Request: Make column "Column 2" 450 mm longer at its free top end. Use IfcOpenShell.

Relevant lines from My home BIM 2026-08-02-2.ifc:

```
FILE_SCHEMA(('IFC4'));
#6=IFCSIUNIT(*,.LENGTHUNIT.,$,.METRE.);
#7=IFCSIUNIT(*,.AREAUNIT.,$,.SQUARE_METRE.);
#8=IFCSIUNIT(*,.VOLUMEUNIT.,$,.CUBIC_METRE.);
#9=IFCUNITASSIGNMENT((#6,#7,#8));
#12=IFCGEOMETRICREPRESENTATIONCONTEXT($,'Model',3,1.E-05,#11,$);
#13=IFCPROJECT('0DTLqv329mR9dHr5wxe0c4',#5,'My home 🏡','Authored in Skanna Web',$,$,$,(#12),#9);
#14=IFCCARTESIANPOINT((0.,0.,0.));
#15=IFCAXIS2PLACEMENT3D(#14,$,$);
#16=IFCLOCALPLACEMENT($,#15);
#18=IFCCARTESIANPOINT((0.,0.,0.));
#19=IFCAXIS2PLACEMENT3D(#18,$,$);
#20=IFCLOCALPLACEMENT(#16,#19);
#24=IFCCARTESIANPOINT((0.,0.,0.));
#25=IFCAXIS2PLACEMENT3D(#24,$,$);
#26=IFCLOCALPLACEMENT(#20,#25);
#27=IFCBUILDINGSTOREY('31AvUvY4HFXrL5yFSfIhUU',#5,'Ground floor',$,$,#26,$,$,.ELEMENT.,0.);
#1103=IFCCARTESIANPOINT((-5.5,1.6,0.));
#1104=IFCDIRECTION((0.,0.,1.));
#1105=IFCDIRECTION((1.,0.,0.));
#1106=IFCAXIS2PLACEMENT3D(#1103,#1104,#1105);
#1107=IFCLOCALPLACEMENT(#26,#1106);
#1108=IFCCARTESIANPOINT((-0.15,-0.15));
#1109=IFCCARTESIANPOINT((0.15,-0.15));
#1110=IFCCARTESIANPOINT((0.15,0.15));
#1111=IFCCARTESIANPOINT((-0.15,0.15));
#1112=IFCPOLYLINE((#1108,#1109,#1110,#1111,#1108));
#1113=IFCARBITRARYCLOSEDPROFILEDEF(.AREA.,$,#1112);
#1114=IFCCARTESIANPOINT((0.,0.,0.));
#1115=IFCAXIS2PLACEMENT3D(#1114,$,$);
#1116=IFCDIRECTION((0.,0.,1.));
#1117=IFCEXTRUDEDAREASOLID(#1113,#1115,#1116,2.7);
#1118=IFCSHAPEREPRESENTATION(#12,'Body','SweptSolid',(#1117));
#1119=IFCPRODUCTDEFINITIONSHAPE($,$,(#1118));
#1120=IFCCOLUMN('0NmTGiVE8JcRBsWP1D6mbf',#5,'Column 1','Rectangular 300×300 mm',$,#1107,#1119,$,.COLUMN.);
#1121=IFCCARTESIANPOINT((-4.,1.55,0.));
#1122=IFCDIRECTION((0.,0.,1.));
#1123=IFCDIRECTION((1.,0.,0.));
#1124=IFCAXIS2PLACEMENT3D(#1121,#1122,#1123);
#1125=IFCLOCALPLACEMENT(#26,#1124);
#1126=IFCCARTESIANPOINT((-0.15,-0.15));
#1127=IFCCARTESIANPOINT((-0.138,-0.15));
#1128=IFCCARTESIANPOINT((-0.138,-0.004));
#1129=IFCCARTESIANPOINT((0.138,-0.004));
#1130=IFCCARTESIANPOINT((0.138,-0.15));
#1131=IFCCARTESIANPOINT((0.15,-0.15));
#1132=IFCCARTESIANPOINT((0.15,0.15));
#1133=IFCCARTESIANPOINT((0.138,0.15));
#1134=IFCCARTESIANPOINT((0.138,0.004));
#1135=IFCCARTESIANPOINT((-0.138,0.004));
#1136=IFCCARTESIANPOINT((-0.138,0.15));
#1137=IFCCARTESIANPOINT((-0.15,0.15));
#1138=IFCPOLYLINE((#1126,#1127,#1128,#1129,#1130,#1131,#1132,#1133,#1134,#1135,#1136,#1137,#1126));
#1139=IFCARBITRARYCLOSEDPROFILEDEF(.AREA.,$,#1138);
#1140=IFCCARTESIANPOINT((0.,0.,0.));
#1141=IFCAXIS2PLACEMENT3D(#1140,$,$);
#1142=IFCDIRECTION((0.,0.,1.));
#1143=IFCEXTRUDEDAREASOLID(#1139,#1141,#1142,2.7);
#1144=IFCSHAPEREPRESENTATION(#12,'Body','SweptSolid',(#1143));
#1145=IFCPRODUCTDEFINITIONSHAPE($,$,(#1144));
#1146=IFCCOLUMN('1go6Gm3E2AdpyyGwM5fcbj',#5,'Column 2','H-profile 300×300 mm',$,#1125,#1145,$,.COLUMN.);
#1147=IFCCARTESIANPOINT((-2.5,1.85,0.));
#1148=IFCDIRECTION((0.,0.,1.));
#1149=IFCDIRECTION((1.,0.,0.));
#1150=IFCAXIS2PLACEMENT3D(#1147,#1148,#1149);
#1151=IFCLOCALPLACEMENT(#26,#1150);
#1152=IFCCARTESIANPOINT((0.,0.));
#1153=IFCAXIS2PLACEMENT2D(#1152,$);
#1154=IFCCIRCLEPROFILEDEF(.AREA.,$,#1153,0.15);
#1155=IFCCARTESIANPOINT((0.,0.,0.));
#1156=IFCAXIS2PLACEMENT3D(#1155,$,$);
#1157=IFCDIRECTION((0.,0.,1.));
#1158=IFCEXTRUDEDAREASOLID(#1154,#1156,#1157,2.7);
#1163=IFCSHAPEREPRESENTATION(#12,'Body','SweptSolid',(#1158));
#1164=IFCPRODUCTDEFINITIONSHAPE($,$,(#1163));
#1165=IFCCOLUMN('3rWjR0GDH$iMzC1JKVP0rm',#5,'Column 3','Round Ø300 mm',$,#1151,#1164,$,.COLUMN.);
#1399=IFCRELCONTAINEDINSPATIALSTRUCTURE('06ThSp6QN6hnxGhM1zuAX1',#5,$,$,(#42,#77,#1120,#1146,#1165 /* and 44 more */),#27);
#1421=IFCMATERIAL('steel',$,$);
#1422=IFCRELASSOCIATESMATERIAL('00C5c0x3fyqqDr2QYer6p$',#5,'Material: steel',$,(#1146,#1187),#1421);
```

```python
import ifcopenshell
import ifcopenshell.util.unit

model = ifcopenshell.open("My home BIM 2026-08-02-2.ifc")
unit_scale = ifcopenshell.util.unit.calculate_unit_scale(model)

member = model.by_id(1146)
change = 0.45 / unit_scale

# The extrusion runs towards the end named, so only its depth changes.
body = next(r for r in member.Representation.Representations if r.RepresentationIdentifier == "Body")
solid = body.Items[0]
old_length = solid.Depth
solid.Depth += change

print(f"length {old_length:g} -> {solid.Depth:g}")

model.write("My home BIM 2026-08-02-2_rev.ifc")
```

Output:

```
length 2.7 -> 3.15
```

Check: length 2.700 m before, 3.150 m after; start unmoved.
